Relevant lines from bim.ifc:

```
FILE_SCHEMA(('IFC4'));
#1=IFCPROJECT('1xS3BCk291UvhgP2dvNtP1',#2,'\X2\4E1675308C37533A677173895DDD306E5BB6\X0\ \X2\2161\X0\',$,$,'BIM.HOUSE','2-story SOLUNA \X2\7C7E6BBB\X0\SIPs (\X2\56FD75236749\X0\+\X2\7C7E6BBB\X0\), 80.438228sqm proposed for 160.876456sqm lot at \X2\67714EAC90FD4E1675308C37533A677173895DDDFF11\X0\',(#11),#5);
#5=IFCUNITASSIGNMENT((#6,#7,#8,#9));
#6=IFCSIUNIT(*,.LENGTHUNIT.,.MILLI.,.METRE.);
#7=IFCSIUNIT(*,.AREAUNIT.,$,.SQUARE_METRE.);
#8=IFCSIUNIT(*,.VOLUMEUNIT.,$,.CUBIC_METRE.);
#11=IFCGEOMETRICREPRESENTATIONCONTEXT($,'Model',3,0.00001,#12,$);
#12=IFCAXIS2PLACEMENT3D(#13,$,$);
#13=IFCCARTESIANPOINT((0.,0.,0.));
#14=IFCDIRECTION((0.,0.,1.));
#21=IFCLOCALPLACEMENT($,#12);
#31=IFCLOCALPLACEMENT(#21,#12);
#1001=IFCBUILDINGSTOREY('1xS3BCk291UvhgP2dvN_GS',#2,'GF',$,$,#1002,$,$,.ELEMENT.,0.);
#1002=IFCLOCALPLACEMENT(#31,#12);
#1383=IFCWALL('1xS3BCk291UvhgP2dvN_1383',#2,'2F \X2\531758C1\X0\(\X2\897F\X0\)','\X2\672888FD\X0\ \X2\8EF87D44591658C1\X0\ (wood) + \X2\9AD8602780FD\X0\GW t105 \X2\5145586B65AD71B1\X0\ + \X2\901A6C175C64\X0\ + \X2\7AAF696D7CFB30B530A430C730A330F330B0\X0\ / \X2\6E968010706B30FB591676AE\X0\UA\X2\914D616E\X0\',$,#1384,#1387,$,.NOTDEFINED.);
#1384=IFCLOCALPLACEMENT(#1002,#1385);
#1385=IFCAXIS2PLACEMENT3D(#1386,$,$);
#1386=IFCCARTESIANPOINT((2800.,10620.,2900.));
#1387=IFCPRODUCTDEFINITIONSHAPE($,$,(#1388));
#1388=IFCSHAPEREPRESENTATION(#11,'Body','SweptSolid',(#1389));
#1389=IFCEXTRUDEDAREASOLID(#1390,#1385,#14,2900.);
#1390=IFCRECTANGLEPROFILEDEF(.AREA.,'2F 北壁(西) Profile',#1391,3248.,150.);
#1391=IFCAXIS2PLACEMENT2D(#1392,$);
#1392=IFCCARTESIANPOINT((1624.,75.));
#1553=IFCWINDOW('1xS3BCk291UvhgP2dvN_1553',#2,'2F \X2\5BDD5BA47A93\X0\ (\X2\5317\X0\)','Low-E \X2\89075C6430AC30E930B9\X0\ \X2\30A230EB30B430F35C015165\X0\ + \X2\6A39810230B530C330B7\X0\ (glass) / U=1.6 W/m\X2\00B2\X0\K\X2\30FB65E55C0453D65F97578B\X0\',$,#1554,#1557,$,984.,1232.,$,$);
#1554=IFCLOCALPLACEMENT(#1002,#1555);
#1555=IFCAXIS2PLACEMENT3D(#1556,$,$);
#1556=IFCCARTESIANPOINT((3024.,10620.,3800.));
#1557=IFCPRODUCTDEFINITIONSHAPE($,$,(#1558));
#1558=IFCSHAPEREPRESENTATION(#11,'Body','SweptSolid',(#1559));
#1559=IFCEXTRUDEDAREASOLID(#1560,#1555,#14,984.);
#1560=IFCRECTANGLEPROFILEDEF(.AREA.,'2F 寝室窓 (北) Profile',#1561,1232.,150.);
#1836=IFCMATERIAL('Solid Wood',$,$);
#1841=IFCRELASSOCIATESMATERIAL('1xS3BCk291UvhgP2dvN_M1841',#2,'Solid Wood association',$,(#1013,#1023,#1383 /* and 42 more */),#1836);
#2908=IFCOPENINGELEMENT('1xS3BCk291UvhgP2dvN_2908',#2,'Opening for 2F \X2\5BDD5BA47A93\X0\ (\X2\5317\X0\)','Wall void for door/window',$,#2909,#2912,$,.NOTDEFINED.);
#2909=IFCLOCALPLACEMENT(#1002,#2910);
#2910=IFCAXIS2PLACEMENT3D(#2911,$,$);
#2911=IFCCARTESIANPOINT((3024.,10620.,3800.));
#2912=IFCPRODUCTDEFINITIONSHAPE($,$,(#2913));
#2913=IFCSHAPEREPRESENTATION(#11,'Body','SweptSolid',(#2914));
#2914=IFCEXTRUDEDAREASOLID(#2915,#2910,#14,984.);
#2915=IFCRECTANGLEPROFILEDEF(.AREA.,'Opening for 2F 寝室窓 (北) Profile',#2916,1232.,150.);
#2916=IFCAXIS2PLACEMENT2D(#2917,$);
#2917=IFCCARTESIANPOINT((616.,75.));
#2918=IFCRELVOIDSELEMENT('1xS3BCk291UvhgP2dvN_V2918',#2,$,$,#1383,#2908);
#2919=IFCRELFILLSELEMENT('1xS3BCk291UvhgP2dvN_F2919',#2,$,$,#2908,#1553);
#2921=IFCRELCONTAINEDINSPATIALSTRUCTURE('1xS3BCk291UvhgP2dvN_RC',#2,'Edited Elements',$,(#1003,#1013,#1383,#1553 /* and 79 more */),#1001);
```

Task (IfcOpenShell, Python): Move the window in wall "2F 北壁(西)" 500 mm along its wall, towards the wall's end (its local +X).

```python
import ifcopenshell
import ifcopenshell.api.geometry
import ifcopenshell.util.placement

model = ifcopenshell.open("bim.ifc")

window = model.by_id(1553)
opening = window.FillsVoids[0].RelatingOpeningElement
wall = opening.VoidsElements[0].RelatingBuildingElement

wall_matrix = ifcopenshell.util.placement.get_local_placement(wall.ObjectPlacement)
shift = wall_matrix[:3, 0] * 500.0
before = ifcopenshell.util.placement.get_local_placement(window.ObjectPlacement)[:3, 3].copy()

# The window is not placed relative to its opening, so move both.
for product in (opening, window):
    matrix = ifcopenshell.util.placement.get_local_placement(product.ObjectPlacement)
    matrix[:3, 3] += shift
    ifcopenshell.api.geometry.edit_object_placement(model, product=product, matrix=matrix, is_si=False)

after = ifcopenshell.util.placement.get_local_placement(window.ObjectPlacement)[:3, 3]
print("window moved by", (after - before).round(3) + 0.0)

model.write("bim-out.ifc")
```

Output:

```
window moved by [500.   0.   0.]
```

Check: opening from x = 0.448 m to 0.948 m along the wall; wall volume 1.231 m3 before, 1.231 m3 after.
